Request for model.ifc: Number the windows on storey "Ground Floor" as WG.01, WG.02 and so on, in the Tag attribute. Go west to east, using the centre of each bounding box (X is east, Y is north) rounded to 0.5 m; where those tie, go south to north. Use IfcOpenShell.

First a look at what the model holds.

```python
import ifcopenshell
import ifcopenshell.util.element
import ifcopenshell.util.placement

model = ifcopenshell.open("model.ifc")
print(model.schema)
storey = next(s for s in model.by_type("IfcBuildingStorey") if s.Name == "Ground Floor")
windows = [e for e in ifcopenshell.util.element.get_decomposition(storey) if e.is_a("IfcWindow")]
for e in sorted(windows, key=lambda e: e.id()):
    origin = ifcopenshell.util.placement.get_local_placement(e.ObjectPlacement)[:3, 3]
    print(e.id(), e.Tag, e.Name, origin.round(2) + 0.0, sep=" | ")
```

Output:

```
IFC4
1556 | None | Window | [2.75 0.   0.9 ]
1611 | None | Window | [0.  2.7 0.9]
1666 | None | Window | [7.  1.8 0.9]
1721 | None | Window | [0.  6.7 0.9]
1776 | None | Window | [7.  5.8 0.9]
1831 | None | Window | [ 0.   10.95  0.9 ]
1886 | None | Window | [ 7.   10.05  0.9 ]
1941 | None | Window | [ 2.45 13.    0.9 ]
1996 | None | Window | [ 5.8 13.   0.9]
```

```python
import ifcopenshell
import ifcopenshell.geom
import ifcopenshell.util.element
import ifcopenshell.util.shape

model = ifcopenshell.open("model.ifc")
settings = ifcopenshell.geom.settings()
settings.set("use-world-coords", True)


def centre(element):
    shape = ifcopenshell.geom.create_shape(settings, element)
    return ifcopenshell.util.shape.get_bbox_centroid(shape.geometry)


storey = next(s for s in model.by_type("IfcBuildingStorey") if s.Name == "Ground Floor")
windows = [e for e in ifcopenshell.util.element.get_decomposition(storey) if e.is_a("IfcWindow")]

# Insertion points can sit at a corner or the storey origin, so sort by the geometry (in metres).
centres = {e: centre(e) for e in windows}
windows.sort(key=lambda e: (round(centres[e][0] / 0.5), centres[e][1]))

for i, e in enumerate(windows, start=1):
    number = f"WG.{i:02d}"
    e.Tag = number
    print(e.id(), number)

model.write("model_rev.ifc")
```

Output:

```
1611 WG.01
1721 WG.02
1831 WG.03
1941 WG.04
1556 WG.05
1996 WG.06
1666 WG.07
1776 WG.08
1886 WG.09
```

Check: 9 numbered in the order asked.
